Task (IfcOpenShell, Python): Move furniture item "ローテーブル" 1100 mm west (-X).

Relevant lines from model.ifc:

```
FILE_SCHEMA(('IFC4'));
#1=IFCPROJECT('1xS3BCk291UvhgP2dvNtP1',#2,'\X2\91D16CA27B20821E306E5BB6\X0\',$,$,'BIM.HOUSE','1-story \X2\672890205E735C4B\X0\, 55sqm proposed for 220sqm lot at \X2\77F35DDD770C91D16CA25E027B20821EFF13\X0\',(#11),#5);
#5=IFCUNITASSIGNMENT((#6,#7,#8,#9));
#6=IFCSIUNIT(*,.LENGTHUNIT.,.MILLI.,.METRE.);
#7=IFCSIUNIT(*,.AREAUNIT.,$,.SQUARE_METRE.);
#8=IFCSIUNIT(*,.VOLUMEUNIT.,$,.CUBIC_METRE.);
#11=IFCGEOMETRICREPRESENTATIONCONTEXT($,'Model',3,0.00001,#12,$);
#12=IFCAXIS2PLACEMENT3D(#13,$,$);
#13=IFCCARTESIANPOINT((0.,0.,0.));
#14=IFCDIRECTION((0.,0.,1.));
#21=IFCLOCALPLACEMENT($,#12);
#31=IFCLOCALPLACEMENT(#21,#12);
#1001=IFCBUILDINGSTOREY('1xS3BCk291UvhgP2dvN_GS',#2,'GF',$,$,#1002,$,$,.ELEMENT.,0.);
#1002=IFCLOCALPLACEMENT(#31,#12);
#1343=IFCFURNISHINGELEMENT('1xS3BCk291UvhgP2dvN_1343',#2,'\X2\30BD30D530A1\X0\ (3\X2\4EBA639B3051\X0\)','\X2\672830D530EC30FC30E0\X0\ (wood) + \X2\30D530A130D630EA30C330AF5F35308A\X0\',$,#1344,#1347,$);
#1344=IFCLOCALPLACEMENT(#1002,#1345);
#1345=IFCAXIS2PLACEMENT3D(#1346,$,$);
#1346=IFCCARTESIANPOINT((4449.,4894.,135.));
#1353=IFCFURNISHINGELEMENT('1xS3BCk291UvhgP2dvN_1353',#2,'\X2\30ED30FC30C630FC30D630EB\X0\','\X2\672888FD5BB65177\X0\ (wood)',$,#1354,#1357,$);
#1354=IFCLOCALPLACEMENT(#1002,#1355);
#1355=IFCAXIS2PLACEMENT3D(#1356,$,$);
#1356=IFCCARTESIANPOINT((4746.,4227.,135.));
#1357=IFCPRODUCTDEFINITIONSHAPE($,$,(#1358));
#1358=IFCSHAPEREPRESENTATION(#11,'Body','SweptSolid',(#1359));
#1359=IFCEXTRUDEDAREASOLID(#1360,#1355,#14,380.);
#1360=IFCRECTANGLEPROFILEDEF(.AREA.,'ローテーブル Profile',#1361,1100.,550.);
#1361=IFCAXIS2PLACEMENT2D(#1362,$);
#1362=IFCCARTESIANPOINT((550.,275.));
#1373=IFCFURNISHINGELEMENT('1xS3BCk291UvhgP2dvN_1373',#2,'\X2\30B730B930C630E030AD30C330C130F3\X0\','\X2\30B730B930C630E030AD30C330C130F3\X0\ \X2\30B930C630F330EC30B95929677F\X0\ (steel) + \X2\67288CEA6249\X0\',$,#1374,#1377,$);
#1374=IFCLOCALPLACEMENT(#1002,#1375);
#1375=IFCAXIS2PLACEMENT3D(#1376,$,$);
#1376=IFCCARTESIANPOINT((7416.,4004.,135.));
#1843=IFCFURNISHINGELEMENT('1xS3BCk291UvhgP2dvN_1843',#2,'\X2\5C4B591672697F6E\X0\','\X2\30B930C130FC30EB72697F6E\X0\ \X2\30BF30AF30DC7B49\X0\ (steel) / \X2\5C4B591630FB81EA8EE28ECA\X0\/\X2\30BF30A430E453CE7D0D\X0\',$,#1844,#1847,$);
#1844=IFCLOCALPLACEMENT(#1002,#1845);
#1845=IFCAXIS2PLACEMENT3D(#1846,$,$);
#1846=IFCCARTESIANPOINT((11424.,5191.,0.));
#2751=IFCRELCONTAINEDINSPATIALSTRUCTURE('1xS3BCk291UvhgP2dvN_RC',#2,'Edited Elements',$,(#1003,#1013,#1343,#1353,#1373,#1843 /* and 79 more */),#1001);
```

```python
import ifcopenshell
import ifcopenshell.api.geometry
import ifcopenshell.util.placement

model = ifcopenshell.open("model.ifc")

item = model.by_guid("1xS3BCk291UvhgP2dvN_1353")
matrix = ifcopenshell.util.placement.get_local_placement(item.ObjectPlacement)
matrix[0, 3] -= 1100.0
ifcopenshell.api.geometry.edit_object_placement(model, product=item, matrix=matrix, is_si=False)

print(ifcopenshell.util.placement.get_local_placement(item.ObjectPlacement).round(3) + 0.0)

model.write("model_rev.ifc")
```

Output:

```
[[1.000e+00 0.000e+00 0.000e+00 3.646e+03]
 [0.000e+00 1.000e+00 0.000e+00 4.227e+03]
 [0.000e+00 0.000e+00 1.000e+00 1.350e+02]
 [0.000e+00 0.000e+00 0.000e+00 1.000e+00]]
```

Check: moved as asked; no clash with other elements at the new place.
